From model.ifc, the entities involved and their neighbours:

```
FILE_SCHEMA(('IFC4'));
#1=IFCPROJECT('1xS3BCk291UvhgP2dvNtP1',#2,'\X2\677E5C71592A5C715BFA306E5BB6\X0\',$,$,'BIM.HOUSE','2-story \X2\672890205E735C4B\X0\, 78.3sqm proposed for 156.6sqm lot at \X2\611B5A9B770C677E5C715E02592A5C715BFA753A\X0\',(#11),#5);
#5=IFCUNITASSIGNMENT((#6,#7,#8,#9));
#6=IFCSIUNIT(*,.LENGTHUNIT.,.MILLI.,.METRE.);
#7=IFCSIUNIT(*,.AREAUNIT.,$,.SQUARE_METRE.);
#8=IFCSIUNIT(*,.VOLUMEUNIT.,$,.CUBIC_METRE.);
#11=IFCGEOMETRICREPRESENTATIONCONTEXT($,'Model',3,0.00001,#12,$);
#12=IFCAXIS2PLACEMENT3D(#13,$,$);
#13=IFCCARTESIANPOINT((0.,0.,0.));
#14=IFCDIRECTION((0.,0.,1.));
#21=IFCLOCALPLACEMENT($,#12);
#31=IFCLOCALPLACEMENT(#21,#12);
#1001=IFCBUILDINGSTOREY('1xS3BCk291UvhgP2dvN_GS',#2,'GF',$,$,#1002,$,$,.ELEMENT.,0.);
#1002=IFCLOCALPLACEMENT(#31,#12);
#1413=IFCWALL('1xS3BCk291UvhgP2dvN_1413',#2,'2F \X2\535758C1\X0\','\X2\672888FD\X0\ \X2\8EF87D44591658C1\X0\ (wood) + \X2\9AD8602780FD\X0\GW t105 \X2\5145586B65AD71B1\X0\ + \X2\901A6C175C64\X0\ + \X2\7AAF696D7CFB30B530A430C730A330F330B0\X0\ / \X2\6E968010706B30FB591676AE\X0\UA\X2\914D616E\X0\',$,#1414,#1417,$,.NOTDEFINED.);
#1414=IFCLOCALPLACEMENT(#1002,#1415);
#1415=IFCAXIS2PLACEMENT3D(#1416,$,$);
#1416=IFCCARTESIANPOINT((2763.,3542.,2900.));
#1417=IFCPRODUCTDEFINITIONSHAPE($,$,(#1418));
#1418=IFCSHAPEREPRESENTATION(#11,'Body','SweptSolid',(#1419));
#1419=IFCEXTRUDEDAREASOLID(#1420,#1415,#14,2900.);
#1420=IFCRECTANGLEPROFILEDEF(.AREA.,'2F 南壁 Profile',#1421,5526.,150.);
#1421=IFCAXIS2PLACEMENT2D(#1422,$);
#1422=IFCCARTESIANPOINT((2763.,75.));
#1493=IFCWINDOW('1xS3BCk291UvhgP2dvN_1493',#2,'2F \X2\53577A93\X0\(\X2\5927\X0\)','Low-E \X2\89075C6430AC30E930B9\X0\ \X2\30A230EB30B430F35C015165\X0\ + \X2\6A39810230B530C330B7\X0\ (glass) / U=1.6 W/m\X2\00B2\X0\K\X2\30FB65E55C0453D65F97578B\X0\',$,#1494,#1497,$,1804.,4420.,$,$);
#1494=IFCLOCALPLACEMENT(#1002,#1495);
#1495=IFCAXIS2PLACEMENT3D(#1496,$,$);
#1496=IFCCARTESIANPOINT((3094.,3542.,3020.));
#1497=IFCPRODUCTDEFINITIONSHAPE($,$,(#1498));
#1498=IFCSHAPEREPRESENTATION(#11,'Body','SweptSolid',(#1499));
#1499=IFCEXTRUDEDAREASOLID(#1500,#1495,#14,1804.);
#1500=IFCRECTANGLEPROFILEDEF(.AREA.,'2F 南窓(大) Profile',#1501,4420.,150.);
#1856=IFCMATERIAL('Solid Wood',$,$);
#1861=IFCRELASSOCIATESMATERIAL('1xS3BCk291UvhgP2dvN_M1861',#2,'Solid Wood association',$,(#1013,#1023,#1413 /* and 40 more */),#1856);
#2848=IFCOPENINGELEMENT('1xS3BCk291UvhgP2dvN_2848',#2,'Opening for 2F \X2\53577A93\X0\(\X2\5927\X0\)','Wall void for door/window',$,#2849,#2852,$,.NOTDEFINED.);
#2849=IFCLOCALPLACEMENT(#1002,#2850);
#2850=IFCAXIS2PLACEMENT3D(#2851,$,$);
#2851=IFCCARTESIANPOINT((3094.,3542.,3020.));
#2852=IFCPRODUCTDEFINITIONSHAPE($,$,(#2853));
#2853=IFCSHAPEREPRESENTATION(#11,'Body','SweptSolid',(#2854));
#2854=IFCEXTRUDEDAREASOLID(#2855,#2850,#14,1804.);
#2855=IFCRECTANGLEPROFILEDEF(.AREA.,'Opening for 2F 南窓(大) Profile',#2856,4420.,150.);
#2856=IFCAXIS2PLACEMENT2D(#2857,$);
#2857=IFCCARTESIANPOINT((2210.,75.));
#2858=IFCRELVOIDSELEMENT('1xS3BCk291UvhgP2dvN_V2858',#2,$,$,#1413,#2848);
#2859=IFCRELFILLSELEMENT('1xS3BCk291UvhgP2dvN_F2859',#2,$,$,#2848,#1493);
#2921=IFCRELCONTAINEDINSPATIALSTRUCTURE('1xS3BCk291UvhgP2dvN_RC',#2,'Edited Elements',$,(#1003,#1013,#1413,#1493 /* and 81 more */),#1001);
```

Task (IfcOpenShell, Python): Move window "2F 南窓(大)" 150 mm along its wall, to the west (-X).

```python
import ifcopenshell
import ifcopenshell.api.geometry
import ifcopenshell.util.placement
import ifcopenshell.util.unit

model = ifcopenshell.open("model.ifc")
unit_scale = ifcopenshell.util.unit.calculate_unit_scale(model)

window = model.by_id(1493)
opening = window.FillsVoids[0].RelatingOpeningElement
wall = opening.VoidsElements[0].RelatingBuildingElement

wall_matrix = ifcopenshell.util.placement.get_local_placement(wall.ObjectPlacement)
shift = wall_matrix[:3, 0] * -0.15 / unit_scale
before = ifcopenshell.util.placement.get_local_placement(window.ObjectPlacement)[:3, 3].copy()

# The window is not placed relative to its opening, so move both.
for product in (opening, window):
    matrix = ifcopenshell.util.placement.get_local_placement(product.ObjectPlacement)
    matrix[:3, 3] += shift
    ifcopenshell.api.geometry.edit_object_placement(model, product=product, matrix=matrix, is_si=False)

after = ifcopenshell.util.placement.get_local_placement(window.ObjectPlacement)[:3, 3]
print("window moved by", (after - before).round(3) + 0.0)

model.write("model_rev.ifc")
```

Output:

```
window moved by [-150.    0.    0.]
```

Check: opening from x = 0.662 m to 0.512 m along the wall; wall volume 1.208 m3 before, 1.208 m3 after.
